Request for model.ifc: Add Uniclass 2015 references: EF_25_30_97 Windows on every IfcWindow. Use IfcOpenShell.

First a look at what the model holds.

```python
import ifcopenshell

model = ifcopenshell.open("model.ifc")
print(model.schema)
print("classifications:", [c.Name for c in model.by_type("IfcClassification")])
for ifc_class in ("IfcDoor", "IfcRoof", "IfcStair", "IfcWall", "IfcWindow"):
    print(ifc_class, len(model.by_type(ifc_class)))
```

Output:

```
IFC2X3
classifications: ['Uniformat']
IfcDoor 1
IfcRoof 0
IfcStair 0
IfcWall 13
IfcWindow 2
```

```python
import ifcopenshell
import ifcopenshell.api.classification

model = ifcopenshell.open("model.ifc")

# IFC2X3 requires Source and Edition and has no link from the project to the system.
system = model.create_entity("IfcClassification", Source="NBS", Edition="2015", Name="Uniclass 2015")

codes = {
    "IfcWindow": ("EF_25_30_97", "Windows"),
}
for ifc_class, (code, name) in codes.items():
    products = model.by_type(ifc_class)
    ifcopenshell.api.classification.add_reference(
        model, products=products, classification=system, identification=code, name=name
    )
    print(code, len(products))

model.write("model-out.ifc")
```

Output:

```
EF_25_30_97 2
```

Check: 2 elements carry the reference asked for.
